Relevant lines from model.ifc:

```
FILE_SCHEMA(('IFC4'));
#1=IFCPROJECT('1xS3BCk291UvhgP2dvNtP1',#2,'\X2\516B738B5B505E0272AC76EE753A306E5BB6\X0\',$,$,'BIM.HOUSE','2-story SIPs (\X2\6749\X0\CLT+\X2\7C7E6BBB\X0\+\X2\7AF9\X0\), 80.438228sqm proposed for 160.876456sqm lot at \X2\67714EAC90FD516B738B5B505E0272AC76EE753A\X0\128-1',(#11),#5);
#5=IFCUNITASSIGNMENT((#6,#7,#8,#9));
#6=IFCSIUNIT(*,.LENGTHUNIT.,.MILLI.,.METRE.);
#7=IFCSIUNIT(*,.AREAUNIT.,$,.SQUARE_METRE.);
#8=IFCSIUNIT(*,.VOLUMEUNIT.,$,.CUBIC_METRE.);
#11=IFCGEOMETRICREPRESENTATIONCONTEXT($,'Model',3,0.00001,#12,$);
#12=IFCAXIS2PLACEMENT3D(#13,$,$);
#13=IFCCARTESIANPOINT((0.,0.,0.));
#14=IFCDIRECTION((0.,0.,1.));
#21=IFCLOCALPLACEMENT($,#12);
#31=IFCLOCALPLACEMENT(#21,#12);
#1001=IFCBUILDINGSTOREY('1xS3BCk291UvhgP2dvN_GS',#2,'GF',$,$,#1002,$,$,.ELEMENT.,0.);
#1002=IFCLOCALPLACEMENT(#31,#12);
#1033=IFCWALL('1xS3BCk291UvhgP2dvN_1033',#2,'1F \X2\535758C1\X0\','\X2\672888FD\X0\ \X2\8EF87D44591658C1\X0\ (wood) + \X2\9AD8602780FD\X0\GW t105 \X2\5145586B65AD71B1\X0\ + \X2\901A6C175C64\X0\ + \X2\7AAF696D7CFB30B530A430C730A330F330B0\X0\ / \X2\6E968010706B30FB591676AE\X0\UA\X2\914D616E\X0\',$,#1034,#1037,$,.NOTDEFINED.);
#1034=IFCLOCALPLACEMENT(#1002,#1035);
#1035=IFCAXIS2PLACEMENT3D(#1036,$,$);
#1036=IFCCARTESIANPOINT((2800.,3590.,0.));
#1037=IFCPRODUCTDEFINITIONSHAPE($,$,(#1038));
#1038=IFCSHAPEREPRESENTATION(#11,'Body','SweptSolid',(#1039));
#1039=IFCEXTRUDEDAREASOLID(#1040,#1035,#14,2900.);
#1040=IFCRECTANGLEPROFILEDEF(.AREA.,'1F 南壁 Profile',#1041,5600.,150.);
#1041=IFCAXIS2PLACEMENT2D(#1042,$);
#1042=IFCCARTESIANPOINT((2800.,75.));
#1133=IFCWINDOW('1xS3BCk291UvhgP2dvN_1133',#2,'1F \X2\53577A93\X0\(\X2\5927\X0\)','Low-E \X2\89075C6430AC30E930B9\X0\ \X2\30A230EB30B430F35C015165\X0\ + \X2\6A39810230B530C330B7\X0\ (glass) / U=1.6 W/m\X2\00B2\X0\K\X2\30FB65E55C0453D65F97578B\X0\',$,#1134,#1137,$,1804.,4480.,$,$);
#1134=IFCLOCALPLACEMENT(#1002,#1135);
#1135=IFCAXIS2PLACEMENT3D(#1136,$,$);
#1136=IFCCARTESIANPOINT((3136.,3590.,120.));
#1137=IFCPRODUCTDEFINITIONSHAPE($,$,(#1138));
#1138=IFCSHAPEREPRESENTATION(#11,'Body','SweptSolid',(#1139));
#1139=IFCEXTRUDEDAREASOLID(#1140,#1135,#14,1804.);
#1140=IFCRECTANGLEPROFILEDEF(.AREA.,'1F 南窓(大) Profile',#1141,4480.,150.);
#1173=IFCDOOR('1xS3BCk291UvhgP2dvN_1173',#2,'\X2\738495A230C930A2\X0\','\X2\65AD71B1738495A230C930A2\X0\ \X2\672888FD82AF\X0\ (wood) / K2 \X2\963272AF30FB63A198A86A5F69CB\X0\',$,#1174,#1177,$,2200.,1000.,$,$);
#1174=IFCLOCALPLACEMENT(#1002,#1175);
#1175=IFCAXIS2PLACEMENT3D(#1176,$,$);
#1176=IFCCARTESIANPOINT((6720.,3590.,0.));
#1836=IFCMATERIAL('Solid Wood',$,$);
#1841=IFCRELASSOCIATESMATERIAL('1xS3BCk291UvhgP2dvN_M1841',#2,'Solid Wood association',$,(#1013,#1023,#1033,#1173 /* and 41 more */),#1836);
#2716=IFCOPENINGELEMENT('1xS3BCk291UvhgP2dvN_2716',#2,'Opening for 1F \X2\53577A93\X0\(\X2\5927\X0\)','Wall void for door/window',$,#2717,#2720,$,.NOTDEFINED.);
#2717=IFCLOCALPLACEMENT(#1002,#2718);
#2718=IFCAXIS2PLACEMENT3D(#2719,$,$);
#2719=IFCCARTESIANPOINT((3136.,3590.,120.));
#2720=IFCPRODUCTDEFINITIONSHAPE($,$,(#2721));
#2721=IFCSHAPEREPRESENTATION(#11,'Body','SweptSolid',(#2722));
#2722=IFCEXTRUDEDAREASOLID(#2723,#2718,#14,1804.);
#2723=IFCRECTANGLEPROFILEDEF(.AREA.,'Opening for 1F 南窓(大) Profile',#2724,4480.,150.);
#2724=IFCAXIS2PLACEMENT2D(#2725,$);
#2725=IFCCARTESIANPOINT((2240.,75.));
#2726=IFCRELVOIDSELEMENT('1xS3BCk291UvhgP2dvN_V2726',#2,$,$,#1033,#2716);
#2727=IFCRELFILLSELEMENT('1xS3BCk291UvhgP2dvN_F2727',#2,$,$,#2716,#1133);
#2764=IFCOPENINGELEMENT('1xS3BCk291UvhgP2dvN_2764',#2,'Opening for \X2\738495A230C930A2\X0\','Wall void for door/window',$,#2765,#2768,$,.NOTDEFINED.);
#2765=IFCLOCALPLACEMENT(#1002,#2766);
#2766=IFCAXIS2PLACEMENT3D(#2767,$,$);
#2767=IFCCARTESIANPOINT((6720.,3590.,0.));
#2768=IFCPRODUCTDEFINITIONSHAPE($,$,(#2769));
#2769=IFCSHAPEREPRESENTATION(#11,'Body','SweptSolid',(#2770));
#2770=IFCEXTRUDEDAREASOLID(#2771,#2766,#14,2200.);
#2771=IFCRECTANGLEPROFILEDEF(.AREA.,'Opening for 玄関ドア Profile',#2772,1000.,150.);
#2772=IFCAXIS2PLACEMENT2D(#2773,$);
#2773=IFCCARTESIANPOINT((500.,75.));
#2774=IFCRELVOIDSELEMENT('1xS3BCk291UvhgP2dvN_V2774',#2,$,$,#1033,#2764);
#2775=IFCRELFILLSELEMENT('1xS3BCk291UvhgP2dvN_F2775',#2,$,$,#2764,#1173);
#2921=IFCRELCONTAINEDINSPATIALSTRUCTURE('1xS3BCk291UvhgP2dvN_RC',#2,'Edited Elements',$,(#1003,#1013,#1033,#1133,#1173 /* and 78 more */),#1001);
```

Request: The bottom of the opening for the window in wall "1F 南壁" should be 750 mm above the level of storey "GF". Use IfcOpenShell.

```python
import numpy as np
import ifcopenshell
import ifcopenshell.api.geometry
import ifcopenshell.geom
import ifcopenshell.util.element
import ifcopenshell.util.placement
import ifcopenshell.util.shape
import ifcopenshell.util.unit

model = ifcopenshell.open("model.ifc")
unit_scale = ifcopenshell.util.unit.calculate_unit_scale(model)

window = model.by_guid("1xS3BCk291UvhgP2dvN_1133")
opening = window.FillsVoids[0].RelatingOpeningElement
storey = ifcopenshell.util.element.get_container(window, ifc_class="IfcBuildingStorey")
level = ifcopenshell.util.placement.get_local_placement(storey.ObjectPlacement)[2, 3]

# The opening's origin need not be at the sill, so measure its lowest point.
shape = ifcopenshell.geom.create_shape(ifcopenshell.geom.settings(), opening)
bottom = ifcopenshell.util.shape.get_shape_bottom_elevation(shape, shape.geometry) / unit_scale
dz = level + 0.75 / unit_scale - bottom

shift = np.array([0.0, 0.0, dz])
# The window is not placed relative to its opening, so move both.
for product in (opening, window):
    matrix = ifcopenshell.util.placement.get_local_placement(product.ObjectPlacement)
    matrix[:3, 3] += shift
    ifcopenshell.api.geometry.edit_object_placement(model, product=product, matrix=matrix, is_si=False)

print(f"moved by {dz * unit_scale:+.3f} m")

model.write("model_v2.ifc")
```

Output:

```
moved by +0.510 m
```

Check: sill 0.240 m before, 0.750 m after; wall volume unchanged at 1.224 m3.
